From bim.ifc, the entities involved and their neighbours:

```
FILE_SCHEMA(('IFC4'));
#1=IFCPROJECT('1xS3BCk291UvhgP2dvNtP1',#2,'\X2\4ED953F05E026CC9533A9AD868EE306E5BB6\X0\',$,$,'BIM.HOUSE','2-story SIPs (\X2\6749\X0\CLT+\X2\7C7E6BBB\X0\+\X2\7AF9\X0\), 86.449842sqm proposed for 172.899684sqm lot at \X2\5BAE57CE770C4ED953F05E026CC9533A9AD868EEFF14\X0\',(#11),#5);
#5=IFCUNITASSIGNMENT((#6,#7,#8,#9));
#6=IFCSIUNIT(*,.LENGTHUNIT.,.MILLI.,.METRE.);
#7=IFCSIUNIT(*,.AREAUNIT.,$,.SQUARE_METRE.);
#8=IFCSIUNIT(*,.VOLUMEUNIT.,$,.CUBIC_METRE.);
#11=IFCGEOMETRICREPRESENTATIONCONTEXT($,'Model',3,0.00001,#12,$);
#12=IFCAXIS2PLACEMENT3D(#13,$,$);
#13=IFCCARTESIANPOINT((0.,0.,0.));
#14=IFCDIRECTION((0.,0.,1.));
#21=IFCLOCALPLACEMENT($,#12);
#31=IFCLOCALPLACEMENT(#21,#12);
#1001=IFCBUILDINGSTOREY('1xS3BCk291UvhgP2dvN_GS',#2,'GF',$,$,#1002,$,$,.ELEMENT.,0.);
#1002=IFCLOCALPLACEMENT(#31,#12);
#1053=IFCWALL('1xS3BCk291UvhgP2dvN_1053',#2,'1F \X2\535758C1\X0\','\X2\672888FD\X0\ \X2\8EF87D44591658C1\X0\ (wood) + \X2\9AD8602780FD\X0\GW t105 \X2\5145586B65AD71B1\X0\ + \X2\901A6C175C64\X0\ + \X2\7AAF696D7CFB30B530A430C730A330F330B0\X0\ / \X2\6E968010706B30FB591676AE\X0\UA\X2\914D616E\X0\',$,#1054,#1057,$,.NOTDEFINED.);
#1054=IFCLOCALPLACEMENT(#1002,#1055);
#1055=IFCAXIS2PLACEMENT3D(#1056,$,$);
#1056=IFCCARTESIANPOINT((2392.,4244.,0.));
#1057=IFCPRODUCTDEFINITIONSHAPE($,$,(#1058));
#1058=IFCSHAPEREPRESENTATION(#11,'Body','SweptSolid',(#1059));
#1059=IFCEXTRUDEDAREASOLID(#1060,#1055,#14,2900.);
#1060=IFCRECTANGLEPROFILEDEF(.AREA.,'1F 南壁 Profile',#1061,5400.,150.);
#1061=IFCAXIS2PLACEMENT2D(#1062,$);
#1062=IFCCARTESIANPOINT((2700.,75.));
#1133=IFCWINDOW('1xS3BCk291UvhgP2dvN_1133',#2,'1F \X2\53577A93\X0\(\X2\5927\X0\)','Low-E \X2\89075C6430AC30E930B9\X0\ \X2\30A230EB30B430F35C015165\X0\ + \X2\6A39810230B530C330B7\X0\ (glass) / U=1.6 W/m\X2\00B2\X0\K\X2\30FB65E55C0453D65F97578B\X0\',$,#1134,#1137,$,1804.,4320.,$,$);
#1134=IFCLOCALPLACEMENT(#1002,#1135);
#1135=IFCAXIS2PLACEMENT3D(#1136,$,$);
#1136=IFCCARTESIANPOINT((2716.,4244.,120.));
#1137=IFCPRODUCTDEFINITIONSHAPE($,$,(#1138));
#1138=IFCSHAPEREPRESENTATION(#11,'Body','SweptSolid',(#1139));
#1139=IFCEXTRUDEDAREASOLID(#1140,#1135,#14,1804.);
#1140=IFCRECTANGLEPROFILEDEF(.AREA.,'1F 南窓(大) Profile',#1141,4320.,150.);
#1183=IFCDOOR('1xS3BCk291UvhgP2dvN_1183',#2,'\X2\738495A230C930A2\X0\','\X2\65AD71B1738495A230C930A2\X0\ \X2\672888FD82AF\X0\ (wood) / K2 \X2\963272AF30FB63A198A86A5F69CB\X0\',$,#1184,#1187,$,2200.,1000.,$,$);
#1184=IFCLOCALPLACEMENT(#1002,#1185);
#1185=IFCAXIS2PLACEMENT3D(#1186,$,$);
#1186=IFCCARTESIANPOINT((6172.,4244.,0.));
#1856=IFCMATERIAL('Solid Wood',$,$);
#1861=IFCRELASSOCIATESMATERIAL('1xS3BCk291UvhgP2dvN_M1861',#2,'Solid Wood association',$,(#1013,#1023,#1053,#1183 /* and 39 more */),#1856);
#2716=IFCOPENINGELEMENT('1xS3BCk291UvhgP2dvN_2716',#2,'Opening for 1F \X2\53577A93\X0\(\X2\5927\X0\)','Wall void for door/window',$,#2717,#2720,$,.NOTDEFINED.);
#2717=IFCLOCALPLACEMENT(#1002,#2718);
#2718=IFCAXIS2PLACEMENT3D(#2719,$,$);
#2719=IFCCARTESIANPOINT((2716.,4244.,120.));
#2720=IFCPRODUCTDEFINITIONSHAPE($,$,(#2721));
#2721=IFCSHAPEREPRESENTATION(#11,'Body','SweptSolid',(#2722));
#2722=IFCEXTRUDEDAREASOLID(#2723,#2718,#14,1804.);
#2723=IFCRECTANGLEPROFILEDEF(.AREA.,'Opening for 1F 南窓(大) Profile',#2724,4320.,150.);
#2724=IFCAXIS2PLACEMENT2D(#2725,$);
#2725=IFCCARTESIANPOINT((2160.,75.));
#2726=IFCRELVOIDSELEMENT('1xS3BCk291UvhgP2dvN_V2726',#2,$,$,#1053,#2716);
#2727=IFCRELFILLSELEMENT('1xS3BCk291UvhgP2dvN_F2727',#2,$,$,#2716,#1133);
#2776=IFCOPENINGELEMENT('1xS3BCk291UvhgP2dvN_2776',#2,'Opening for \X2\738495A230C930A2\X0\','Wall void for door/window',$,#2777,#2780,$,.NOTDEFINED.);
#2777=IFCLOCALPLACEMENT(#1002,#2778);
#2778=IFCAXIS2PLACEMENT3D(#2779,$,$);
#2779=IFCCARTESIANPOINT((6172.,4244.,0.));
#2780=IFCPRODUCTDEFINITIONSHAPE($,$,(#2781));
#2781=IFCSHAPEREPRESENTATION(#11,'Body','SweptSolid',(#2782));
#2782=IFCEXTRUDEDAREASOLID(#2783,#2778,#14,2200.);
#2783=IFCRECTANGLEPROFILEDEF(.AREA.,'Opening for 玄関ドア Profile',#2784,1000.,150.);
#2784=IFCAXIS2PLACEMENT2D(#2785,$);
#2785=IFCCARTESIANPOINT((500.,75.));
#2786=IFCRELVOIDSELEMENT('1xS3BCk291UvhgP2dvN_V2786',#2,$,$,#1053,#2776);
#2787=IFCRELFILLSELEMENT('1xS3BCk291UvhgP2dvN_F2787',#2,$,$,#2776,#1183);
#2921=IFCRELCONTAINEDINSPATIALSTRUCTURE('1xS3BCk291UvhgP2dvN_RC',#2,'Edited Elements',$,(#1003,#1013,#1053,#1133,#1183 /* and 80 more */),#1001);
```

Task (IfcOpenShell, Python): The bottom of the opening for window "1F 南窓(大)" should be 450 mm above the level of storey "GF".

```python
import numpy as np
import ifcopenshell
import ifcopenshell.api.geometry
import ifcopenshell.geom
import ifcopenshell.util.element
import ifcopenshell.util.placement
import ifcopenshell.util.shape
import ifcopenshell.util.unit

model = ifcopenshell.open("bim.ifc")
unit_scale = ifcopenshell.util.unit.calculate_unit_scale(model)

window = model.by_guid("1xS3BCk291UvhgP2dvN_1133")
opening = window.FillsVoids[0].RelatingOpeningElement
storey = ifcopenshell.util.element.get_container(window, ifc_class="IfcBuildingStorey")
level = ifcopenshell.util.placement.get_local_placement(storey.ObjectPlacement)[2, 3]

# The opening's origin need not be at the sill, so measure its lowest point.
shape = ifcopenshell.geom.create_shape(ifcopenshell.geom.settings(), opening)
bottom = ifcopenshell.util.shape.get_shape_bottom_elevation(shape, shape.geometry) / unit_scale
dz = level + 450.0 - bottom

shift = np.array([0.0, 0.0, dz])
# The window is not placed relative to its opening, so move both.
for product in (opening, window):
    matrix = ifcopenshell.util.placement.get_local_placement(product.ObjectPlacement)
    matrix[:3, 3] += shift
    ifcopenshell.api.geometry.edit_object_placement(model, product=product, matrix=matrix, is_si=False)

print(f"moved by {dz * unit_scale:+.3f} m")

model.write("bim_rev.ifc")
```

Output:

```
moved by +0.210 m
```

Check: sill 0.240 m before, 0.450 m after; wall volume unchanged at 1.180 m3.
